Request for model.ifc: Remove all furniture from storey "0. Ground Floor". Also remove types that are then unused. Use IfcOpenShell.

First a look at what the model holds.

```python
import ifcopenshell
import ifcopenshell.util.element

model = ifcopenshell.open("model.ifc")
print(model.schema)
storey = next(s for s in model.by_type("IfcBuildingStorey") if s.Name == "0. Ground Floor")
furniture = [e for e in ifcopenshell.util.element.get_decomposition(storey) if e.is_a("IfcFurnishingElement")]
seen = {}
for e in furniture:
    element_type = ifcopenshell.util.element.get_type(e)
    name = element_type.Name if element_type not in (None, e) else None
    seen[name] = seen.get(name, 0) + 1
for name, count in sorted(seen.items(), key=str):
    print(count, "x", name)
```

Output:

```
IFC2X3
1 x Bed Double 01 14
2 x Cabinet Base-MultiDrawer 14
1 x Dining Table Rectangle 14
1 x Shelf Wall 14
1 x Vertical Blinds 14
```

```python
import ifcopenshell
import ifcopenshell.api.root
import ifcopenshell.util.element

model = ifcopenshell.open("model.ifc")

storey = next(s for s in model.by_type("IfcBuildingStorey") if s.Name == "0. Ground Floor")
furniture = [e for e in ifcopenshell.util.element.get_decomposition(storey) if e.is_a("IfcFurnishingElement")]
types = {ifcopenshell.util.element.get_type(e) for e in furniture} - {None, *furniture}

for e in furniture:
    ifcopenshell.api.root.remove_product(model, product=e)
print(len(furniture), "removed")

unused = [t for t in types if not ifcopenshell.util.element.get_types(t)]
for t in unused:
    ifcopenshell.api.root.remove_product(model, product=t)
print(len(unused), "unused types removed")

model.write("model_updated.ifc")
```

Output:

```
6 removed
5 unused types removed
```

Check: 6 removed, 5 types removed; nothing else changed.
